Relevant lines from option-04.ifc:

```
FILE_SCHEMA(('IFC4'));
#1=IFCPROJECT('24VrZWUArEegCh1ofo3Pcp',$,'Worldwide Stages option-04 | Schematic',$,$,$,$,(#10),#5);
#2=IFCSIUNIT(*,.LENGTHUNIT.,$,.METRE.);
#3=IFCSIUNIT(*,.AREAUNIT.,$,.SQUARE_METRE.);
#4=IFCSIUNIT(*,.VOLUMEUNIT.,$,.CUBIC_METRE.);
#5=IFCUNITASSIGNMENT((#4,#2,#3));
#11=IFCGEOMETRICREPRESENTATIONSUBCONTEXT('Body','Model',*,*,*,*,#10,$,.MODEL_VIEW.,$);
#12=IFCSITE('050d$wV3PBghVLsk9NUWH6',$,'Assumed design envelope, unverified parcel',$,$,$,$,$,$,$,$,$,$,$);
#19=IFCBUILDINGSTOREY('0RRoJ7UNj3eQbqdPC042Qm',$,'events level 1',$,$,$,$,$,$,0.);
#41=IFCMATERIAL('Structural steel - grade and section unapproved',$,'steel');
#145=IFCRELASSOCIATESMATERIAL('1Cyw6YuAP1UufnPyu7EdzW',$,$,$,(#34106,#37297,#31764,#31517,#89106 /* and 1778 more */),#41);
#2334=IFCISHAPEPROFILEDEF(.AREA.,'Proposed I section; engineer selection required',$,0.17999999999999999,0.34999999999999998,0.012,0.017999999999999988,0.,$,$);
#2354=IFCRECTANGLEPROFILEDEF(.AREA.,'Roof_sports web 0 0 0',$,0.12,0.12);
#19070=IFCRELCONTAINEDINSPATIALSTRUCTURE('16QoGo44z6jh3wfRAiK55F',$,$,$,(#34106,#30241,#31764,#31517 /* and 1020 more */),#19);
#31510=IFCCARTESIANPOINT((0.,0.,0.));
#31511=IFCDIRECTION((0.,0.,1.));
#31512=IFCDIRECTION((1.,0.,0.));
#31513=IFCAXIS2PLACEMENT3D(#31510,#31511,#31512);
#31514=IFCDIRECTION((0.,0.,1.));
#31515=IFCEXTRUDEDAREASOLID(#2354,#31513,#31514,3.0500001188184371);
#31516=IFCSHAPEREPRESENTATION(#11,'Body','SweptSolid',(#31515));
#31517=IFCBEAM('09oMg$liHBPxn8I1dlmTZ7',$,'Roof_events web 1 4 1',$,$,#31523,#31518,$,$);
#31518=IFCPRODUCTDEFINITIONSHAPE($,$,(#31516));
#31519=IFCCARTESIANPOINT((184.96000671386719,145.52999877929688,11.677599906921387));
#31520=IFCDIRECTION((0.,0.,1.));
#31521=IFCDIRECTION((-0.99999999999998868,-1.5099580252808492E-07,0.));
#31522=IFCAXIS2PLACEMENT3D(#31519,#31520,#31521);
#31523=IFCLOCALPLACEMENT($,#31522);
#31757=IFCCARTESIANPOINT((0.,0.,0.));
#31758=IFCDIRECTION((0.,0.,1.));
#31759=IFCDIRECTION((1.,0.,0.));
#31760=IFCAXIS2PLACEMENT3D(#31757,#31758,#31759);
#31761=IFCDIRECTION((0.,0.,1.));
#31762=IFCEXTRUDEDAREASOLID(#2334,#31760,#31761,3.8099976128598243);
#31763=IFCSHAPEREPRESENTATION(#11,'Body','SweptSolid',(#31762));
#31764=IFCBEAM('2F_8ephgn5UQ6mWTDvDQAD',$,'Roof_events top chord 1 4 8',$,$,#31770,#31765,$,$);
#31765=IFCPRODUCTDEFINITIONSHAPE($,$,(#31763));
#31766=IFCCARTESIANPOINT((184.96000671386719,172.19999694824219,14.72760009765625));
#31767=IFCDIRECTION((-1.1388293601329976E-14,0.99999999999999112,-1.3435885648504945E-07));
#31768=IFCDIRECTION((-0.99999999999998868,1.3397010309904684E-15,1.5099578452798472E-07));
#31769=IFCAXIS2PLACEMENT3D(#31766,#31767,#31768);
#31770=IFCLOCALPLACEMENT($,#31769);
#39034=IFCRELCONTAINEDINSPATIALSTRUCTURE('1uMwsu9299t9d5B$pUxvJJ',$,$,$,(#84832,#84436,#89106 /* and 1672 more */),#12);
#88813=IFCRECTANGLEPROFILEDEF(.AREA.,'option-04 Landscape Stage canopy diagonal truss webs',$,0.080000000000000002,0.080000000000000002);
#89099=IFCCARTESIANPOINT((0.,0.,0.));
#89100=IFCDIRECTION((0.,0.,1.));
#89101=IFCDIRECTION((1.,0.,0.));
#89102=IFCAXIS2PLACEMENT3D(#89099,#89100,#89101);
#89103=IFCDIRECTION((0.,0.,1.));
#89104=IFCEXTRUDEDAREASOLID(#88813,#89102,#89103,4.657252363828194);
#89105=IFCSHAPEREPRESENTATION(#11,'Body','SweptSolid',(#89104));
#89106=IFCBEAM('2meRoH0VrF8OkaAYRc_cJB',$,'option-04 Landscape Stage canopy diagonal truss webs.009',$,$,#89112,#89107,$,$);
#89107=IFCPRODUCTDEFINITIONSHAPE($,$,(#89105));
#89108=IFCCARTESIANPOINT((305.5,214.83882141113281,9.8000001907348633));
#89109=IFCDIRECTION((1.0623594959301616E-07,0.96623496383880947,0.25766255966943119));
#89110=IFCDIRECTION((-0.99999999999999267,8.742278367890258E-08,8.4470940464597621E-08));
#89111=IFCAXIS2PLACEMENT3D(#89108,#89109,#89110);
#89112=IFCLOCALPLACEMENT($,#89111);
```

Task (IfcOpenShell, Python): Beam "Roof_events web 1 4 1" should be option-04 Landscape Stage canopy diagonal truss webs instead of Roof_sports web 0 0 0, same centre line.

```python
import ifcopenshell
import ifcopenshell.util.element
import ifcopenshell.util.representation

model = ifcopenshell.open("option-04.ifc")

member = model.by_guid("09oMg$liHBPxn8I1dlmTZ7")
source = next(p for p in model.by_type("IfcRectangleProfileDef") if p.ProfileName == "option-04 Landscape Stage canopy diagonal truss webs")

body = ifcopenshell.util.representation.get_representation(member, "Model", "Body")
solid = body.Items[0]
old_profile = solid.SweptArea

# Copy the section's sizes but keep this member's own profile position.
profile = ifcopenshell.util.element.copy(model, source)
profile.Position = old_profile.Position
solid.SweptArea = profile
if not model.get_total_inverses(old_profile):
    ifcopenshell.util.element.remove_deep2(model, old_profile)

print(solid.SweptArea)

model.write("option-04_updated.ifc")
```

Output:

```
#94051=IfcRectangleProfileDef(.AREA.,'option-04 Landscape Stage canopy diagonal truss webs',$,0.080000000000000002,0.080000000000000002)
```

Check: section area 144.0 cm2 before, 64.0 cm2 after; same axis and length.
